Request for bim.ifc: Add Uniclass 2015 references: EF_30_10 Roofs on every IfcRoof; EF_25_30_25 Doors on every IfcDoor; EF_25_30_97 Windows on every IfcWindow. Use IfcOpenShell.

First a look at what the model holds.

```python
import ifcopenshell

model = ifcopenshell.open("bim.ifc")
print(model.schema)
print("classifications:", [c.Name for c in model.by_type("IfcClassification")])
for ifc_class in ("IfcDoor", "IfcRoof", "IfcStair", "IfcWall", "IfcWindow"):
    print(ifc_class, len(model.by_type(ifc_class)))
```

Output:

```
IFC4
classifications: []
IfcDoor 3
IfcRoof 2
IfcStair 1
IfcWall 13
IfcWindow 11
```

```python
import ifcopenshell
import ifcopenshell.api.classification

model = ifcopenshell.open("bim.ifc")

system = ifcopenshell.api.classification.add_classification(model, classification="Uniclass 2015")

codes = {
    "IfcRoof": ("EF_30_10", "Roofs"),
    "IfcDoor": ("EF_25_30_25", "Doors"),
    "IfcWindow": ("EF_25_30_97", "Windows"),
}
for ifc_class, (code, name) in codes.items():
    products = model.by_type(ifc_class)
    ifcopenshell.api.classification.add_reference(
        model, products=products, classification=system, identification=code, name=name
    )
    print(code, len(products))

model.write("bim_updated.ifc")
```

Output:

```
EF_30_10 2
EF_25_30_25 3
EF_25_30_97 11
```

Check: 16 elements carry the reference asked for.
